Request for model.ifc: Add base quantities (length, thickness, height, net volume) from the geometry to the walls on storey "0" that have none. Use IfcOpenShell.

First a look at what the model holds.

```python
import ifcopenshell
import ifcopenshell.util.element
import ifcopenshell.util.unit

model = ifcopenshell.open("model.ifc")
print(model.schema)
for unit_type in ("LENGTHUNIT", "AREAUNIT", "VOLUMEUNIT"):
    print(unit_type, ifcopenshell.util.unit.calculate_unit_scale(model, unit_type))
storey = next(s for s in model.by_type("IfcBuildingStorey") if s.Name == "0")
walls = [e for e in ifcopenshell.util.element.get_decomposition(storey) if e.is_a("IfcWall")]
for e in sorted(walls, key=lambda e: e.id()):
    print(e.id(), e.is_a(), e.Name, list(ifcopenshell.util.element.get_psets(e, qtos_only=True)), sep=" | ")
```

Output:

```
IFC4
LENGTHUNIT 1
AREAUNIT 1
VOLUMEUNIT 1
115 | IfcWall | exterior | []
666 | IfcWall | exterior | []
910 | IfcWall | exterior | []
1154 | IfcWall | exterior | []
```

```python
import ifcopenshell
import ifcopenshell.api.pset
import ifcopenshell.geom
import ifcopenshell.util.element
import ifcopenshell.util.shape
import ifcopenshell.util.unit

model = ifcopenshell.open("model.ifc")
unit_scale = ifcopenshell.util.unit.calculate_unit_scale(model)
volume_scale = ifcopenshell.util.unit.calculate_unit_scale(model, "VOLUMEUNIT")
settings = ifcopenshell.geom.settings()

storey = next(s for s in model.by_type("IfcBuildingStorey") if s.Name == "0")
walls = [e for e in ifcopenshell.util.element.get_decomposition(storey) if e.is_a("IfcWall")]

for e in sorted(walls, key=lambda e: e.id()):
    if ifcopenshell.util.element.get_psets(e, qtos_only=True, should_inherit=False):
        continue
    # Geometry comes back in metres, in the element's own axes.
    shape = ifcopenshell.geom.create_shape(settings, e)
    values = {
        "Length": ifcopenshell.util.shape.get_x(shape.geometry) / unit_scale,
        "Width": ifcopenshell.util.shape.get_y(shape.geometry) / unit_scale,
        "Height": ifcopenshell.util.shape.get_z(shape.geometry) / unit_scale,
        "NetVolume": ifcopenshell.util.shape.get_volume(shape.geometry) / volume_scale,
    }
    qto = ifcopenshell.api.pset.add_qto(model, product=e, name="Qto_WallBaseQuantities")
    ifcopenshell.api.pset.edit_qto(model, qto=qto, properties=values)
    print(e.id(), {k: round(v, 3) for k, v in values.items()})

model.write("model_edited.ifc")
```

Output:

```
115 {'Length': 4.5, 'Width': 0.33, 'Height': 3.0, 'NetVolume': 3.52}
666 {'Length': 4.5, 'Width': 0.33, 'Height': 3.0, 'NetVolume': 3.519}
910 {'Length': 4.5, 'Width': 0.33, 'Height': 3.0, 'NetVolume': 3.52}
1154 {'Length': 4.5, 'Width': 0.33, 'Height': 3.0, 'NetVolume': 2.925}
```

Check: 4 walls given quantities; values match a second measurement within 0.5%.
